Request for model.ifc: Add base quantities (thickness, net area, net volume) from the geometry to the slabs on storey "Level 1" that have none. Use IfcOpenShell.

First a look at what the model holds.

```python
import ifcopenshell
import ifcopenshell.util.element
import ifcopenshell.util.unit

model = ifcopenshell.open("model.ifc")
print(model.schema)
for unit_type in ("LENGTHUNIT", "AREAUNIT", "VOLUMEUNIT"):
    print(unit_type, ifcopenshell.util.unit.calculate_unit_scale(model, unit_type))
storey = next(s for s in model.by_type("IfcBuildingStorey") if s.Name == "Level 1")
slabs = [e for e in ifcopenshell.util.element.get_decomposition(storey) if e.is_a("IfcSlab")]
for e in sorted(slabs, key=lambda e: e.id()):
    print(e.id(), e.is_a(), e.Name, list(ifcopenshell.util.element.get_psets(e, qtos_only=True)), sep=" | ")
```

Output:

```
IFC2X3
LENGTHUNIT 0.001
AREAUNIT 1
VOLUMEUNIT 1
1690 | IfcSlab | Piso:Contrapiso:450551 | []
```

```python
import ifcopenshell
import ifcopenshell.api.pset
import ifcopenshell.geom
import ifcopenshell.util.element
import ifcopenshell.util.shape
import ifcopenshell.util.unit

model = ifcopenshell.open("model.ifc")
unit_scale = ifcopenshell.util.unit.calculate_unit_scale(model)
area_scale = ifcopenshell.util.unit.calculate_unit_scale(model, "AREAUNIT")
volume_scale = ifcopenshell.util.unit.calculate_unit_scale(model, "VOLUMEUNIT")
settings = ifcopenshell.geom.settings()

storey = next(s for s in model.by_type("IfcBuildingStorey") if s.Name == "Level 1")
slabs = [e for e in ifcopenshell.util.element.get_decomposition(storey) if e.is_a("IfcSlab")]

for e in sorted(slabs, key=lambda e: e.id()):
    if ifcopenshell.util.element.get_psets(e, qtos_only=True, should_inherit=False):
        continue
    # Geometry comes back in metres, in the element's own axes.
    shape = ifcopenshell.geom.create_shape(settings, e)
    values = {
        "Width": ifcopenshell.util.shape.get_z(shape.geometry) / unit_scale,
        "NetArea": ifcopenshell.util.shape.get_footprint_area(shape.geometry) / area_scale,
        "NetVolume": ifcopenshell.util.shape.get_volume(shape.geometry) / volume_scale,
    }
    qto = ifcopenshell.api.pset.add_qto(model, product=e, name="BaseQuantities")
    ifcopenshell.api.pset.edit_qto(model, qto=qto, properties=values)
    print(e.id(), {k: round(v, 3) for k, v in values.items()})

model.write("model_edited.ifc")
```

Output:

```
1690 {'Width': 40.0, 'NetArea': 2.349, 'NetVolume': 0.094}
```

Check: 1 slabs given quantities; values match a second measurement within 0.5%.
